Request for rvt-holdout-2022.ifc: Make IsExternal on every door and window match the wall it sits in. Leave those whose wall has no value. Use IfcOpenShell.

First a look at what the model holds.

```python
import ifcopenshell
import ifcopenshell.util.element

model = ifcopenshell.open("rvt-holdout-2022.ifc")
print(model.schema)
seen = {}
for e in model.by_type("IfcDoor") + model.by_type("IfcWindow"):
    if not e.FillsVoids:
        continue
    host = e.FillsVoids[0].RelatingOpeningElement.VoidsElements[0].RelatingBuildingElement
    own = ifcopenshell.util.element.get_pset(e, f"Pset_{e.is_a()[3:].removesuffix('StandardCase')}Common", "IsExternal")
    wall = ifcopenshell.util.element.get_pset(host, "Pset_WallCommon", "IsExternal")
    seen[e.is_a(), own, wall] = seen.get((e.is_a(), own, wall), 0) + 1
for (cls, own, wall), count in sorted(seen.items(), key=str):
    print(count, cls, "IsExternal:", own, "| host wall:", wall)
```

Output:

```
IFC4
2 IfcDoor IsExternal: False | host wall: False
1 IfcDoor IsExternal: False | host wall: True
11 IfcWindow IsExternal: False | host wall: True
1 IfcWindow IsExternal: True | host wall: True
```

```python
import ifcopenshell
import ifcopenshell.api.pset
import ifcopenshell.util.element

model = ifcopenshell.open("rvt-holdout-2022.ifc")

count = 0
for ifc_class, pset_name in (("IfcDoor", "Pset_DoorCommon"), ("IfcWindow", "Pset_WindowCommon")):
    for e in model.by_type(ifc_class):
        if not e.FillsVoids:
            continue
        host = e.FillsVoids[0].RelatingOpeningElement.VoidsElements[0].RelatingBuildingElement
        external = ifcopenshell.util.element.get_pset(host, "Pset_WallCommon", "IsExternal")
        if external is None or ifcopenshell.util.element.get_pset(e, pset_name, "IsExternal") == external:
            continue
        pset = ifcopenshell.api.pset.add_pset(model, product=e, name=pset_name)
        ifcopenshell.api.pset.edit_pset(model, pset=pset, properties={"IsExternal": external})
        count += 1

print(count, "updated")

model.write("rvt-holdout-2022_rev.ifc")
```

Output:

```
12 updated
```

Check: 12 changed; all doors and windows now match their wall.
